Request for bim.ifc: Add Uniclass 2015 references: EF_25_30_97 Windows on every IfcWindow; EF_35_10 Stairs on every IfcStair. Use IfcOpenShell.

First a look at what the model holds.

```python
import ifcopenshell

model = ifcopenshell.open("bim.ifc")
print(model.schema)
print("classifications:", [c.Name for c in model.by_type("IfcClassification")])
for ifc_class in ("IfcDoor", "IfcRoof", "IfcStair", "IfcWall", "IfcWindow"):
    print(ifc_class, len(model.by_type(ifc_class)))
```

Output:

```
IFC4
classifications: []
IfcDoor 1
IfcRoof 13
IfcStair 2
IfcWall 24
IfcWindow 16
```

```python
import ifcopenshell
import ifcopenshell.api.classification

model = ifcopenshell.open("bim.ifc")

system = ifcopenshell.api.classification.add_classification(model, classification="Uniclass 2015")

codes = {
    "IfcWindow": ("EF_25_30_97", "Windows"),
    "IfcStair": ("EF_35_10", "Stairs"),
}
for ifc_class, (code, name) in codes.items():
    products = model.by_type(ifc_class)
    ifcopenshell.api.classification.add_reference(
        model, products=products, classification=system, identification=code, name=name
    )
    print(code, len(products))

model.write("bim_updated.ifc")
```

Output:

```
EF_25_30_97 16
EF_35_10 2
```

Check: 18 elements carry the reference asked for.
